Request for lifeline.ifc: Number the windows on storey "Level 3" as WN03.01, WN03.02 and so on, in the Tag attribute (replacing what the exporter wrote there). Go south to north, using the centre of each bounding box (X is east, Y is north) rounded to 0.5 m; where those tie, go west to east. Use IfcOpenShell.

First a look at what the model holds.

```python
import ifcopenshell
import ifcopenshell.util.element
import ifcopenshell.util.placement

model = ifcopenshell.open("lifeline.ifc")
print(model.schema)
storey = next(s for s in model.by_type("IfcBuildingStorey") if s.Name == "Level 3")
windows = [e for e in ifcopenshell.util.element.get_decomposition(storey) if e.is_a("IfcWindow")]
for e in sorted(windows, key=lambda e: e.id()):
    origin = ifcopenshell.util.placement.get_local_placement(e.ObjectPlacement)[:3, 3]
    print(e.id(), e.Tag, e.Name, origin.round(2) + 0.0, sep=" | ")
```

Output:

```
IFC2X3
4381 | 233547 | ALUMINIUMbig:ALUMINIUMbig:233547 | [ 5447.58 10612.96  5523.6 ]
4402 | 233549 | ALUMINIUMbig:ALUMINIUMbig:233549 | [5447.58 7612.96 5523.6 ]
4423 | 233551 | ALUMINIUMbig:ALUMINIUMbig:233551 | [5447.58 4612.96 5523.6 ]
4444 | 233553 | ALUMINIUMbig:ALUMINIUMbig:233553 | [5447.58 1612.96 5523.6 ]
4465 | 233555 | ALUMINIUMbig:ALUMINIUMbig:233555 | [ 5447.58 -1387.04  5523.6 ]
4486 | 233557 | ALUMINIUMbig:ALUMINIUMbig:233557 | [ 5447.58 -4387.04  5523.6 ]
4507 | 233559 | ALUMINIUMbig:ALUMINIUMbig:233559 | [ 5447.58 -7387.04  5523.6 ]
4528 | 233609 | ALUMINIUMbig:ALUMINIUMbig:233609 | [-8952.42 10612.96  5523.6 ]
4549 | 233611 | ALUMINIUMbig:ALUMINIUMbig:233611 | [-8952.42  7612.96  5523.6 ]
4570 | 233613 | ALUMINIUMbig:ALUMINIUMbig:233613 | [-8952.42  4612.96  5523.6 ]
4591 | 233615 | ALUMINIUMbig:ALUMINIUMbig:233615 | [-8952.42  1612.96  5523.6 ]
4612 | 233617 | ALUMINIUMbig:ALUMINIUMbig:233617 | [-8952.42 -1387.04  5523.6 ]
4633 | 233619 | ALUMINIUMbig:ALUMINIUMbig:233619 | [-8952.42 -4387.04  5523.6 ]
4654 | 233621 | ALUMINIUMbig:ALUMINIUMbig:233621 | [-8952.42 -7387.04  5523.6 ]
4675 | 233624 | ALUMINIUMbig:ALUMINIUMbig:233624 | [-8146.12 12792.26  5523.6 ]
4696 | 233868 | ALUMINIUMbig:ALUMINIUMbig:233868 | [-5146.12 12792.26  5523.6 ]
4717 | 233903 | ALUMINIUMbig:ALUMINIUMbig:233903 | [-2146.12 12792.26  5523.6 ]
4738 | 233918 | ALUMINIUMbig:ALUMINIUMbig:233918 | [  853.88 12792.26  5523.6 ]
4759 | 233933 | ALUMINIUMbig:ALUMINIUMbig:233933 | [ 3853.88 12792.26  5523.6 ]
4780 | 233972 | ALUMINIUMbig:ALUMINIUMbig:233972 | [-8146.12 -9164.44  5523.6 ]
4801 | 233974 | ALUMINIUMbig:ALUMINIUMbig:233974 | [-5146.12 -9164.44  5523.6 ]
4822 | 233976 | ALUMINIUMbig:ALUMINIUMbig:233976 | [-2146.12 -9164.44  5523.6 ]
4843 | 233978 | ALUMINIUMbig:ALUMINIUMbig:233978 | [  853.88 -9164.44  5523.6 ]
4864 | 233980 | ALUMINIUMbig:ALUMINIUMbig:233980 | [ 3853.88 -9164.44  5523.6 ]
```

```python
import ifcopenshell
import ifcopenshell.geom
import ifcopenshell.util.element
import ifcopenshell.util.shape

model = ifcopenshell.open("lifeline.ifc")
settings = ifcopenshell.geom.settings()
settings.set("use-world-coords", True)


def centre(element):
    shape = ifcopenshell.geom.create_shape(settings, element)
    return ifcopenshell.util.shape.get_bbox_centroid(shape.geometry)


storey = next(s for s in model.by_type("IfcBuildingStorey") if s.Name == "Level 3")
windows = [e for e in ifcopenshell.util.element.get_decomposition(storey) if e.is_a("IfcWindow")]

# Insertion points can sit at a corner or the storey origin, so sort by the geometry (in metres).
centres = {e: centre(e) for e in windows}
windows.sort(key=lambda e: (round(centres[e][1] / 0.5), centres[e][0]))

for i, e in enumerate(windows, start=1):
    number = f"WN03.{i:02d}"
    e.Tag = number
    print(e.id(), number)

model.write("lifeline_edited.ifc")
```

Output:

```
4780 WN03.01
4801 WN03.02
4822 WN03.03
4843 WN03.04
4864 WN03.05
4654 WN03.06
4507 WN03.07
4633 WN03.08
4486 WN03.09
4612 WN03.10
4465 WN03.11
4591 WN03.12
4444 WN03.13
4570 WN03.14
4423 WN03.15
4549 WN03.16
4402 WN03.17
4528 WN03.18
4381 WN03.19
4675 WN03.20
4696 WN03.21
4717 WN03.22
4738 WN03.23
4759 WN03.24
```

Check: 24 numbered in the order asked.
